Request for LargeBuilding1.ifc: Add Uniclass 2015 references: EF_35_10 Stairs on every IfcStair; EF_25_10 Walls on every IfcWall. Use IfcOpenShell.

First a look at what the model holds.

```python
import ifcopenshell

model = ifcopenshell.open("LargeBuilding1.ifc")
print(model.schema)
print("classifications:", [c.Name for c in model.by_type("IfcClassification")])
for ifc_class in ("IfcDoor", "IfcRoof", "IfcStair", "IfcWall", "IfcWindow"):
    print(ifc_class, len(model.by_type(ifc_class)))
```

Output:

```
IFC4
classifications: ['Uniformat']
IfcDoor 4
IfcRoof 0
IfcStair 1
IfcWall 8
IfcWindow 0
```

```python
import ifcopenshell
import ifcopenshell.api.classification

model = ifcopenshell.open("LargeBuilding1.ifc")

system = ifcopenshell.api.classification.add_classification(model, classification="Uniclass 2015")

codes = {
    "IfcStair": ("EF_35_10", "Stairs"),
    "IfcWall": ("EF_25_10", "Walls"),
}
for ifc_class, (code, name) in codes.items():
    products = model.by_type(ifc_class)
    ifcopenshell.api.classification.add_reference(
        model, products=products, classification=system, identification=code, name=name
    )
    print(code, len(products))

model.write("LargeBuilding1_edited.ifc")
```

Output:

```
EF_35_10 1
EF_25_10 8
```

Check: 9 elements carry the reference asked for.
